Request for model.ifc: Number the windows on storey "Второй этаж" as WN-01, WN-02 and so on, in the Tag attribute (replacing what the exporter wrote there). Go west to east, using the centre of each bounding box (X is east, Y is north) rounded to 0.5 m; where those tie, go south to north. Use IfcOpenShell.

First a look at what the model holds.

```python
import ifcopenshell
import ifcopenshell.util.element
import ifcopenshell.util.placement

model = ifcopenshell.open("model.ifc")
print(model.schema)
storey = next(s for s in model.by_type("IfcBuildingStorey") if s.Name == "Второй этаж")
windows = [e for e in ifcopenshell.util.element.get_decomposition(storey) if e.is_a("IfcWindow")]
for e in sorted(windows, key=lambda e: e.id()):
    origin = ifcopenshell.util.placement.get_local_placement(e.ObjectPlacement)[:3, 3]
    print(e.id(), e.Tag, e.Name, origin.round(2) + 0.0, sep=" | ")
```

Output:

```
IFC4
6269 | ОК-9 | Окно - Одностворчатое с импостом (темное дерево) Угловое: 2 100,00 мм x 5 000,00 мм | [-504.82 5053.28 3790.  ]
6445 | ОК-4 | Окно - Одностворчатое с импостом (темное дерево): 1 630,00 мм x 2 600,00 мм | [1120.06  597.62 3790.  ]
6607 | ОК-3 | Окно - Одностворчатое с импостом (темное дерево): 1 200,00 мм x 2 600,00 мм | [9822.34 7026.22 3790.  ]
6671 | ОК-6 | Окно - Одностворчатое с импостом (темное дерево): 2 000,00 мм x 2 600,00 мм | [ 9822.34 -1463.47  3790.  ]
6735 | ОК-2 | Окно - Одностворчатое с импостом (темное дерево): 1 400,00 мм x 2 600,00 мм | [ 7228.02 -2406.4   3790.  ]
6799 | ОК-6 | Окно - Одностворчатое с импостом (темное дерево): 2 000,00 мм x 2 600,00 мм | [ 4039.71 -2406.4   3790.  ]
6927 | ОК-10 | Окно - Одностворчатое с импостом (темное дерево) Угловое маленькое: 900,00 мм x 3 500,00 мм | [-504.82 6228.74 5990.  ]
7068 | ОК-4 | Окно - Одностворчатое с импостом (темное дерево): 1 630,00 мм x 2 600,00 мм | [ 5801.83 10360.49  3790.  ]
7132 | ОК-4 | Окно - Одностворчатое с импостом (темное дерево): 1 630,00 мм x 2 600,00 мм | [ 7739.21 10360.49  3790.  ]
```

```python
import ifcopenshell
import ifcopenshell.geom
import ifcopenshell.util.element
import ifcopenshell.util.shape

model = ifcopenshell.open("model.ifc")
settings = ifcopenshell.geom.settings()
settings.set("use-world-coords", True)


def centre(element):
    shape = ifcopenshell.geom.create_shape(settings, element)
    return ifcopenshell.util.shape.get_bbox_centroid(shape.geometry)


storey = next(s for s in model.by_type("IfcBuildingStorey") if s.Name == "Второй этаж")
windows = [e for e in ifcopenshell.util.element.get_decomposition(storey) if e.is_a("IfcWindow")]

# Insertion points can sit at a corner or the storey origin, so sort by the geometry (in metres).
centres = {e: centre(e) for e in windows}
windows.sort(key=lambda e: (round(centres[e][0] / 0.5), centres[e][1]))

for i, e in enumerate(windows, start=1):
    number = f"WN-{i:02d}"
    e.Tag = number
    print(e.id(), number)

model.write("model_v2.ifc")
```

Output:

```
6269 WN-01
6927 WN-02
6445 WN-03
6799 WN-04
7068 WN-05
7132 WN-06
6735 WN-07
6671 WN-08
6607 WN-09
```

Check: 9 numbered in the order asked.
